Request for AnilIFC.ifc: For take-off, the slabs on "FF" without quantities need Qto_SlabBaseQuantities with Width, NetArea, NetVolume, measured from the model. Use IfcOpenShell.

First a look at what the model holds.

```python
import ifcopenshell
import ifcopenshell.util.element
import ifcopenshell.util.unit

model = ifcopenshell.open("AnilIFC.ifc")
print(model.schema)
for unit_type in ("LENGTHUNIT", "AREAUNIT", "VOLUMEUNIT"):
    print(unit_type, ifcopenshell.util.unit.calculate_unit_scale(model, unit_type))
storey = next(s for s in model.by_type("IfcBuildingStorey") if s.Name == "FF")
slabs = [e for e in ifcopenshell.util.element.get_decomposition(storey) if e.is_a("IfcSlab")]
for e in sorted(slabs, key=lambda e: e.id()):
    print(e.id(), e.is_a(), e.Name, list(ifcopenshell.util.element.get_psets(e, qtos_only=True)), sep=" | ")
```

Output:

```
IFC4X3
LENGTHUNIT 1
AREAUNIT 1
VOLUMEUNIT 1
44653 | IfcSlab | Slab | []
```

```python
import ifcopenshell
import ifcopenshell.api.pset
import ifcopenshell.geom
import ifcopenshell.util.element
import ifcopenshell.util.shape
import ifcopenshell.util.unit

model = ifcopenshell.open("AnilIFC.ifc")
unit_scale = ifcopenshell.util.unit.calculate_unit_scale(model)
area_scale = ifcopenshell.util.unit.calculate_unit_scale(model, "AREAUNIT")
volume_scale = ifcopenshell.util.unit.calculate_unit_scale(model, "VOLUMEUNIT")
settings = ifcopenshell.geom.settings()

storey = next(s for s in model.by_type("IfcBuildingStorey") if s.Name == "FF")
slabs = [e for e in ifcopenshell.util.element.get_decomposition(storey) if e.is_a("IfcSlab")]

for e in sorted(slabs, key=lambda e: e.id()):
    if ifcopenshell.util.element.get_psets(e, qtos_only=True, should_inherit=False):
        continue
    # Geometry comes back in metres, in the element's own axes.
    shape = ifcopenshell.geom.create_shape(settings, e)
    values = {
        "Width": ifcopenshell.util.shape.get_z(shape.geometry) / unit_scale,
        "NetArea": ifcopenshell.util.shape.get_footprint_area(shape.geometry) / area_scale,
        "NetVolume": ifcopenshell.util.shape.get_volume(shape.geometry) / volume_scale,
    }
    qto = ifcopenshell.api.pset.add_qto(model, product=e, name="Qto_SlabBaseQuantities")
    ifcopenshell.api.pset.edit_qto(model, qto=qto, properties=values)
    print(e.id(), {k: round(v, 3) for k, v in values.items()})

model.write("AnilIFC_v2.ifc")
```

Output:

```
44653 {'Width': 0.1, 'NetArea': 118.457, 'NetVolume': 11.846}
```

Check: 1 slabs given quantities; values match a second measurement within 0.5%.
